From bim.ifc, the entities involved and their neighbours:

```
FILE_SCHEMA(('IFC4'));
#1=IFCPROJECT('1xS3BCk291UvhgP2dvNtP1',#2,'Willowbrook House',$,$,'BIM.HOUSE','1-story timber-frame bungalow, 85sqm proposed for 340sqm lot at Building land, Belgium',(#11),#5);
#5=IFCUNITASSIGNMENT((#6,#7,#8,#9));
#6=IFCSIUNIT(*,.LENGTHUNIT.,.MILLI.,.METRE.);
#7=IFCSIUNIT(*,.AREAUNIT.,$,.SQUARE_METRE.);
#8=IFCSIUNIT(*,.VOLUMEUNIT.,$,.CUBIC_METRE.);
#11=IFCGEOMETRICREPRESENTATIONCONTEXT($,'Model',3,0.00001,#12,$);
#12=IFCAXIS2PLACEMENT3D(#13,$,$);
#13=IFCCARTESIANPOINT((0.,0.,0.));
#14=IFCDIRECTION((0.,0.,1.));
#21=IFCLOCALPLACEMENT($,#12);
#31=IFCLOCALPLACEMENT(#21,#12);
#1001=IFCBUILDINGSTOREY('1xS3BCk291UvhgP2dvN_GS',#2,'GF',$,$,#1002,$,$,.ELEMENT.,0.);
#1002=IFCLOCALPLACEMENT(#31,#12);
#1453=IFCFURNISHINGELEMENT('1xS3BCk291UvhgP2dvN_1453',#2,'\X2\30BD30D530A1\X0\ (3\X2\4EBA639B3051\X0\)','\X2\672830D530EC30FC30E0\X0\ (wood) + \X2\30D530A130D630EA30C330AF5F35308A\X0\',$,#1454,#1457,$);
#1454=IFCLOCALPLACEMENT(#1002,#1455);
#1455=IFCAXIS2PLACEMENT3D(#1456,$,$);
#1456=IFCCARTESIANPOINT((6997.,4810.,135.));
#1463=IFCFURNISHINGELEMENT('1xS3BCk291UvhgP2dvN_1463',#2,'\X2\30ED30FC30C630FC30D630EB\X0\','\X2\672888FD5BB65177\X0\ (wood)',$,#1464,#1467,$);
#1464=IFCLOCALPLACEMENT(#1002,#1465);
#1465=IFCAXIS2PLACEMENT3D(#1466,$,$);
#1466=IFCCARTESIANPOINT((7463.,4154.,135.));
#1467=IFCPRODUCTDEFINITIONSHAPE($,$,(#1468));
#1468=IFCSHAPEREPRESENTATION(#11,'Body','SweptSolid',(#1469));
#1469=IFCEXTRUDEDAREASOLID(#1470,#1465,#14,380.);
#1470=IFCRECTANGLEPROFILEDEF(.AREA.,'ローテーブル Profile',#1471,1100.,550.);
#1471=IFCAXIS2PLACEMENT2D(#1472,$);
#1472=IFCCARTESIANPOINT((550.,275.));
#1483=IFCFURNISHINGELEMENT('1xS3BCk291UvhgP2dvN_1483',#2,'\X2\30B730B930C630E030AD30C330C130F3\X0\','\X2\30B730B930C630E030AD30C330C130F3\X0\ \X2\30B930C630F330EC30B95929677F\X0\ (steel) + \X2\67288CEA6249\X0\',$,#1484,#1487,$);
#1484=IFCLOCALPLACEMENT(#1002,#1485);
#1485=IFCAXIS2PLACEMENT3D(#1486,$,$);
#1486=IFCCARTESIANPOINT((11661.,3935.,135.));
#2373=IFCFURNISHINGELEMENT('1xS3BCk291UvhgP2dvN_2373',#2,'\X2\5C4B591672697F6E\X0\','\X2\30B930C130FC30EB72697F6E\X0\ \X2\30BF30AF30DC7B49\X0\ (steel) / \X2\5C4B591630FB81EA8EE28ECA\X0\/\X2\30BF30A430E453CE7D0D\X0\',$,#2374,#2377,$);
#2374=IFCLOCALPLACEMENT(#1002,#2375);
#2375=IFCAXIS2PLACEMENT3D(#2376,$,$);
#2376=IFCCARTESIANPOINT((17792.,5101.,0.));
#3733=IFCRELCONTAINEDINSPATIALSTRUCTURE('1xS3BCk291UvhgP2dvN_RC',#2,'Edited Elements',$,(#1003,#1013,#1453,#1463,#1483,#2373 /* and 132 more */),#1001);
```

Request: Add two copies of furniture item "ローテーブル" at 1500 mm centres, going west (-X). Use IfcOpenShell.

```python
import numpy as np
import ifcopenshell
import ifcopenshell.api.geometry
import ifcopenshell.api.root
import ifcopenshell.util.element
import ifcopenshell.util.placement
import ifcopenshell.util.unit

model = ifcopenshell.open("bim.ifc")
unit_scale = ifcopenshell.util.unit.calculate_unit_scale(model)


def reuse_history(source, copy):
    """copy_class also copies each property set's owner history, people and application; keep the originals."""
    for rel in copy.IsDefinedBy:
        if rel.is_a("IfcRelDefinesByProperties") and (history := rel.RelatingPropertyDefinition.OwnerHistory):
            rel.RelatingPropertyDefinition.OwnerHistory = source.OwnerHistory
            ifcopenshell.util.element.remove_deep2(model, history)


source = model.by_id(1463)
base = ifcopenshell.util.placement.get_local_placement(source.ObjectPlacement)
step = np.array([-1.0, 0.0, 0.0]) * 1.5 / unit_scale

for i in range(1, 3):
    copy = ifcopenshell.api.root.copy_class(model, product=source)
    copy.Representation = ifcopenshell.util.element.copy_deep(
        model, source.Representation, exclude=["IfcGeometricRepresentationContext", "IfcRepresentationMap"]
    )
    reuse_history(source, copy)
    matrix = base.copy()
    matrix[:3, 3] += i * step
    print("added at", matrix[:3, 3].round(3) + 0.0)
    ifcopenshell.api.geometry.edit_object_placement(model, product=copy, matrix=matrix, is_si=False)

model.write("bim_v2.ifc")
```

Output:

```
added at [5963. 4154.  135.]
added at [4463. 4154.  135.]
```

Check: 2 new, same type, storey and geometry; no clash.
